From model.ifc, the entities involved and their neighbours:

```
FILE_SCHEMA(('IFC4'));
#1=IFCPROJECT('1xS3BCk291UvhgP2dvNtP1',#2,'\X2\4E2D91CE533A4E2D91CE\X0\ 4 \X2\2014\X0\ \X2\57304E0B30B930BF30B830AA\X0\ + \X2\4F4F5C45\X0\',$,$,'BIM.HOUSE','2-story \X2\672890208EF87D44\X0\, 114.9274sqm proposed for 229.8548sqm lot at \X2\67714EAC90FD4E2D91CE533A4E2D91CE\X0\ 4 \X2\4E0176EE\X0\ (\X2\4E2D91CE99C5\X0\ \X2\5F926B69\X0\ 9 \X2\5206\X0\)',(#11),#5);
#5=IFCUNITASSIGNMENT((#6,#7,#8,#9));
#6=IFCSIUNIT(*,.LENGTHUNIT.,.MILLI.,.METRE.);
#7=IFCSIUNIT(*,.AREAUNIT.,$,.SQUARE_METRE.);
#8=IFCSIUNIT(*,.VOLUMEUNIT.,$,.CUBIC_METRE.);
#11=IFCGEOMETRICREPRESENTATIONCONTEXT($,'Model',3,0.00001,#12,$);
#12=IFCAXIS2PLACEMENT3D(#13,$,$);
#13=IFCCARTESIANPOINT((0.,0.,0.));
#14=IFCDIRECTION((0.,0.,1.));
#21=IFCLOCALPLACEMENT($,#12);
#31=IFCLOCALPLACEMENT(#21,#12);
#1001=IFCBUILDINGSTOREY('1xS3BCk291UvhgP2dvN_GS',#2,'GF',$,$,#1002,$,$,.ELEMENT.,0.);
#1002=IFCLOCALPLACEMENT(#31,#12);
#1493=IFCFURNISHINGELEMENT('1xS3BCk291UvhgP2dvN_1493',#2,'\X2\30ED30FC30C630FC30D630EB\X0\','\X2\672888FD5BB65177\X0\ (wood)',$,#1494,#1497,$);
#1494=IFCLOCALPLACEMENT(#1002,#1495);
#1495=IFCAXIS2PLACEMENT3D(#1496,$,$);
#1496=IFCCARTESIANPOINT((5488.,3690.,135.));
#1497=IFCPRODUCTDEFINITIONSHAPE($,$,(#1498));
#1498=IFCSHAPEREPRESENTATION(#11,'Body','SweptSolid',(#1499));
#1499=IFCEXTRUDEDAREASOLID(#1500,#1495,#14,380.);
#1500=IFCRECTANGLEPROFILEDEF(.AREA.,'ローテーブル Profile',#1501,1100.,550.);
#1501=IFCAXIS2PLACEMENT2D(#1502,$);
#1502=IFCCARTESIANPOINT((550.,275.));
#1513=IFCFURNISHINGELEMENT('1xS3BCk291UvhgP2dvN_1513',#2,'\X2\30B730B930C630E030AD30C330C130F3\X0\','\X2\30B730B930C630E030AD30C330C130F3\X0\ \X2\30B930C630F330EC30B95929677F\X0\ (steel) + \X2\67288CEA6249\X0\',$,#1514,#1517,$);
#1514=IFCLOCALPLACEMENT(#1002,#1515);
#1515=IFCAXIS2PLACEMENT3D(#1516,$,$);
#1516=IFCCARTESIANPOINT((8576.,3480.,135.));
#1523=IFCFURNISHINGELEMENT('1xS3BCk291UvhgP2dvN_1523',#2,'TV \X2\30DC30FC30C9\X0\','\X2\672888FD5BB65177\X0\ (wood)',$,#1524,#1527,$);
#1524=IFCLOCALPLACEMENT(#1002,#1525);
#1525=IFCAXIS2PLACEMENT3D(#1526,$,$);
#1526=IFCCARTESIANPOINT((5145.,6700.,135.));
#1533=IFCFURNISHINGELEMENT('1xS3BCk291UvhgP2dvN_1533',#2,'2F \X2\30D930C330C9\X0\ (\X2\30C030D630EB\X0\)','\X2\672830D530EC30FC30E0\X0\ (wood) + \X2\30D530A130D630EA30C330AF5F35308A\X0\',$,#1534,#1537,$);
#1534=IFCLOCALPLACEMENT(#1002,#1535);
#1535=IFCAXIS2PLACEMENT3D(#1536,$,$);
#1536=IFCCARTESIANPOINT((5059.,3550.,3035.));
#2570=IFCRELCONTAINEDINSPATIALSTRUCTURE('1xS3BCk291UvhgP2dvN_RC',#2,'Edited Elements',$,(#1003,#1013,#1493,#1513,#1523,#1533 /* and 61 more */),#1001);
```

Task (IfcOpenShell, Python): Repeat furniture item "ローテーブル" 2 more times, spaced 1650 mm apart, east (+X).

```python
import numpy as np
import ifcopenshell
import ifcopenshell.api.geometry
import ifcopenshell.api.root
import ifcopenshell.util.element
import ifcopenshell.util.placement
import ifcopenshell.util.unit

model = ifcopenshell.open("model.ifc")
unit_scale = ifcopenshell.util.unit.calculate_unit_scale(model)


def reuse_history(source, copy):
    """copy_class also copies each property set's owner history, people and application; keep the originals."""
    for rel in copy.IsDefinedBy:
        if rel.is_a("IfcRelDefinesByProperties") and (history := rel.RelatingPropertyDefinition.OwnerHistory):
            rel.RelatingPropertyDefinition.OwnerHistory = source.OwnerHistory
            ifcopenshell.util.element.remove_deep2(model, history)


source = model.by_guid("1xS3BCk291UvhgP2dvN_1493")
base = ifcopenshell.util.placement.get_local_placement(source.ObjectPlacement)
step = np.array([1.0, 0.0, 0.0]) * 1.65 / unit_scale

for i in range(1, 3):
    copy = ifcopenshell.api.root.copy_class(model, product=source)
    copy.Representation = ifcopenshell.util.element.copy_deep(
        model, source.Representation, exclude=["IfcGeometricRepresentationContext", "IfcRepresentationMap"]
    )
    reuse_history(source, copy)
    matrix = base.copy()
    matrix[:3, 3] += i * step
    print("added at", matrix[:3, 3].round(3) + 0.0)
    ifcopenshell.api.geometry.edit_object_placement(model, product=copy, matrix=matrix, is_si=False)

model.write("model_rev.ifc")
```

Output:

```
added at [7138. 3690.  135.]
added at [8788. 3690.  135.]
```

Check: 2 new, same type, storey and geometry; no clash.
